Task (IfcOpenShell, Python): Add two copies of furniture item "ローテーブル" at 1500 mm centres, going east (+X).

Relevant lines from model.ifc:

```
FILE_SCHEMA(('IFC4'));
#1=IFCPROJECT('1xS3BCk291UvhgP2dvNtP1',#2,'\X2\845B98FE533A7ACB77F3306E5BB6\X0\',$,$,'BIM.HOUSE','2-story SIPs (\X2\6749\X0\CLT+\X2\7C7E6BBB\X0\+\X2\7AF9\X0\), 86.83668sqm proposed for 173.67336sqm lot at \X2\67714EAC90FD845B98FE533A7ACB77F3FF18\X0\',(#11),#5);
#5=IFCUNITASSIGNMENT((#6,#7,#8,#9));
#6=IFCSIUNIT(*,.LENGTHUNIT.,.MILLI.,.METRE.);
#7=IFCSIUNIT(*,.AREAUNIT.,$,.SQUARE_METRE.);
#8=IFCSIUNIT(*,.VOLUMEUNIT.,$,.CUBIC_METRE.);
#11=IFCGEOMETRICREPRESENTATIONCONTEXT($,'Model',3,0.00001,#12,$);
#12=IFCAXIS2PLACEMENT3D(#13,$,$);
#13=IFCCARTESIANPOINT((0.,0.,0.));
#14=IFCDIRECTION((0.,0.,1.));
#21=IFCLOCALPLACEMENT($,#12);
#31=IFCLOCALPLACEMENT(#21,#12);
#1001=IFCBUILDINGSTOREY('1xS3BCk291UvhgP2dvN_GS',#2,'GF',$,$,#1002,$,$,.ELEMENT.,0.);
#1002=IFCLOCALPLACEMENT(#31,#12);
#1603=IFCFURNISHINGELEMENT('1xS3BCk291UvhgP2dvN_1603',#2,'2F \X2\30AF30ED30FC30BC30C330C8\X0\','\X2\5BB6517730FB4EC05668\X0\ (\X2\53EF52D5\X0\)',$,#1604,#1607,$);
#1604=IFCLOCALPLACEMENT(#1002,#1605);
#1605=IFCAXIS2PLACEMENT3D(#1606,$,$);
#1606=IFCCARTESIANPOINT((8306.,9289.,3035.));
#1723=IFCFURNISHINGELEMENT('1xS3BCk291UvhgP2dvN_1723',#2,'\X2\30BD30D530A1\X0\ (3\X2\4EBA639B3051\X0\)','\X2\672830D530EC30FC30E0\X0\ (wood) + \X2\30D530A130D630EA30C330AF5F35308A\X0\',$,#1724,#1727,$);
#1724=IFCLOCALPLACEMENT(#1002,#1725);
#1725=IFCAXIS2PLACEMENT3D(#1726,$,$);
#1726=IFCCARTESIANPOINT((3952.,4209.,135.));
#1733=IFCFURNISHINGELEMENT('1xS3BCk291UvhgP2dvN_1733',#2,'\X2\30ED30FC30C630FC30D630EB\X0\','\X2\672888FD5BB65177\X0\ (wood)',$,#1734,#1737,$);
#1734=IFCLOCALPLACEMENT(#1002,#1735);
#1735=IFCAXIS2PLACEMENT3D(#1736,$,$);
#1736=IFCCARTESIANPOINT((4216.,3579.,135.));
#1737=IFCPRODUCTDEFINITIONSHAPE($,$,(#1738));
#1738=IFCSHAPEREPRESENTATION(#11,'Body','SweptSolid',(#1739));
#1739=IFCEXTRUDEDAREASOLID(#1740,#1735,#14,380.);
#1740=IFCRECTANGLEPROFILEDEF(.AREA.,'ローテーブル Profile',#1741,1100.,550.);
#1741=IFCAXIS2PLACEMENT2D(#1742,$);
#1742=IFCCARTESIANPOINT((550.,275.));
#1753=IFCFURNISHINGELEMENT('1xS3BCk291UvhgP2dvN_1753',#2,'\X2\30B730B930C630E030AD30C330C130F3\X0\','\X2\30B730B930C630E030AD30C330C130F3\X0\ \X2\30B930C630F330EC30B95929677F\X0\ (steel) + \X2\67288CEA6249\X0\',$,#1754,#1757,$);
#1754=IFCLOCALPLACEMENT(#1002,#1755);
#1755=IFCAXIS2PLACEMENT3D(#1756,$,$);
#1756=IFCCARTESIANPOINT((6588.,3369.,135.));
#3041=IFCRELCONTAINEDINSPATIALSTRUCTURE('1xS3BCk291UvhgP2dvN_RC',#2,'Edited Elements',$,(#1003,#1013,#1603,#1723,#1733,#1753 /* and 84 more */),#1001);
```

```python
import numpy as np
import ifcopenshell
import ifcopenshell.api.geometry
import ifcopenshell.api.root
import ifcopenshell.util.element
import ifcopenshell.util.placement
import ifcopenshell.util.unit

model = ifcopenshell.open("model.ifc")
unit_scale = ifcopenshell.util.unit.calculate_unit_scale(model)


def reuse_history(source, copy):
    """copy_class also copies each property set's owner history, people and application; keep the originals."""
    for rel in copy.IsDefinedBy:
        if rel.is_a("IfcRelDefinesByProperties") and (history := rel.RelatingPropertyDefinition.OwnerHistory):
            rel.RelatingPropertyDefinition.OwnerHistory = source.OwnerHistory
            ifcopenshell.util.element.remove_deep2(model, history)


source = model.by_guid("1xS3BCk291UvhgP2dvN_1733")
base = ifcopenshell.util.placement.get_local_placement(source.ObjectPlacement)
step = np.array([1.0, 0.0, 0.0]) * 1.5 / unit_scale

for i in range(1, 3):
    copy = ifcopenshell.api.root.copy_class(model, product=source)
    copy.Representation = ifcopenshell.util.element.copy_deep(
        model, source.Representation, exclude=["IfcGeometricRepresentationContext", "IfcRepresentationMap"]
    )
    reuse_history(source, copy)
    matrix = base.copy()
    matrix[:3, 3] += i * step
    print("added at", matrix[:3, 3].round(3) + 0.0)
    ifcopenshell.api.geometry.edit_object_placement(model, product=copy, matrix=matrix, is_si=False)

model.write("model_rev.ifc")
```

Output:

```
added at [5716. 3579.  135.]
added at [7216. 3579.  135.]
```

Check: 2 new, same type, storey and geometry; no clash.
